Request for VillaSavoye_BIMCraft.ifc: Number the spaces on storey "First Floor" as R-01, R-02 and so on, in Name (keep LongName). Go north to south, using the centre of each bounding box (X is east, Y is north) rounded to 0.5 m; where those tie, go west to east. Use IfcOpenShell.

First a look at what the model holds.

```python
import ifcopenshell
import ifcopenshell.util.element
import ifcopenshell.util.placement

model = ifcopenshell.open("VillaSavoye_BIMCraft.ifc")
print(model.schema)
storey = next(s for s in model.by_type("IfcBuildingStorey") if s.Name == "First Floor")
spaces = [e for e in ifcopenshell.util.element.get_decomposition(storey) if e.is_a("IfcSpace")]
for e in sorted(spaces, key=lambda e: e.id()):
    origin = ifcopenshell.util.placement.get_local_placement(e.ObjectPlacement)[:3, 3]
    print(e.id(), e.Name, e.LongName, origin.round(2) + 0.0, sep=" | ")
```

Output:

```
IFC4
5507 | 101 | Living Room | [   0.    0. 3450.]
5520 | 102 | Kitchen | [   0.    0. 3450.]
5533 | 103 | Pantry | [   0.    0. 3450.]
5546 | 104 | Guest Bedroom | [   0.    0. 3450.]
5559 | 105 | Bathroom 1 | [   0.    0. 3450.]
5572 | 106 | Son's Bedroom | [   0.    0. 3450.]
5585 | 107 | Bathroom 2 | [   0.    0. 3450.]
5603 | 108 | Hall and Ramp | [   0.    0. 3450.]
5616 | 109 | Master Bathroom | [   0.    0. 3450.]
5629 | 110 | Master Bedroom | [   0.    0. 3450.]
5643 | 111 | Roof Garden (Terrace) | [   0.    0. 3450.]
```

```python
import ifcopenshell
import ifcopenshell.geom
import ifcopenshell.util.element
import ifcopenshell.util.shape

model = ifcopenshell.open("VillaSavoye_BIMCraft.ifc")
settings = ifcopenshell.geom.settings()
settings.set("use-world-coords", True)


def centre(element):
    shape = ifcopenshell.geom.create_shape(settings, element)
    return ifcopenshell.util.shape.get_bbox_centroid(shape.geometry)


storey = next(s for s in model.by_type("IfcBuildingStorey") if s.Name == "First Floor")
spaces = [e for e in ifcopenshell.util.element.get_decomposition(storey) if e.is_a("IfcSpace")]

# Insertion points can sit at a corner or the storey origin, so sort by the geometry (in metres).
centres = {e: centre(e) for e in spaces}
spaces.sort(key=lambda e: (-round(centres[e][1] / 0.5), centres[e][0]))

for i, e in enumerate(spaces, start=1):
    number = f"R-{i:02d}"
    e.Name = number
    print(e.id(), number)

model.write("VillaSavoye_BIMCraft_edited.ifc")
```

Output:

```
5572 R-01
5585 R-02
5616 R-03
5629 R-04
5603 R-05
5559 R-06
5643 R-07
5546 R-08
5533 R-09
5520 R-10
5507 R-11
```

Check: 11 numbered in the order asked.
